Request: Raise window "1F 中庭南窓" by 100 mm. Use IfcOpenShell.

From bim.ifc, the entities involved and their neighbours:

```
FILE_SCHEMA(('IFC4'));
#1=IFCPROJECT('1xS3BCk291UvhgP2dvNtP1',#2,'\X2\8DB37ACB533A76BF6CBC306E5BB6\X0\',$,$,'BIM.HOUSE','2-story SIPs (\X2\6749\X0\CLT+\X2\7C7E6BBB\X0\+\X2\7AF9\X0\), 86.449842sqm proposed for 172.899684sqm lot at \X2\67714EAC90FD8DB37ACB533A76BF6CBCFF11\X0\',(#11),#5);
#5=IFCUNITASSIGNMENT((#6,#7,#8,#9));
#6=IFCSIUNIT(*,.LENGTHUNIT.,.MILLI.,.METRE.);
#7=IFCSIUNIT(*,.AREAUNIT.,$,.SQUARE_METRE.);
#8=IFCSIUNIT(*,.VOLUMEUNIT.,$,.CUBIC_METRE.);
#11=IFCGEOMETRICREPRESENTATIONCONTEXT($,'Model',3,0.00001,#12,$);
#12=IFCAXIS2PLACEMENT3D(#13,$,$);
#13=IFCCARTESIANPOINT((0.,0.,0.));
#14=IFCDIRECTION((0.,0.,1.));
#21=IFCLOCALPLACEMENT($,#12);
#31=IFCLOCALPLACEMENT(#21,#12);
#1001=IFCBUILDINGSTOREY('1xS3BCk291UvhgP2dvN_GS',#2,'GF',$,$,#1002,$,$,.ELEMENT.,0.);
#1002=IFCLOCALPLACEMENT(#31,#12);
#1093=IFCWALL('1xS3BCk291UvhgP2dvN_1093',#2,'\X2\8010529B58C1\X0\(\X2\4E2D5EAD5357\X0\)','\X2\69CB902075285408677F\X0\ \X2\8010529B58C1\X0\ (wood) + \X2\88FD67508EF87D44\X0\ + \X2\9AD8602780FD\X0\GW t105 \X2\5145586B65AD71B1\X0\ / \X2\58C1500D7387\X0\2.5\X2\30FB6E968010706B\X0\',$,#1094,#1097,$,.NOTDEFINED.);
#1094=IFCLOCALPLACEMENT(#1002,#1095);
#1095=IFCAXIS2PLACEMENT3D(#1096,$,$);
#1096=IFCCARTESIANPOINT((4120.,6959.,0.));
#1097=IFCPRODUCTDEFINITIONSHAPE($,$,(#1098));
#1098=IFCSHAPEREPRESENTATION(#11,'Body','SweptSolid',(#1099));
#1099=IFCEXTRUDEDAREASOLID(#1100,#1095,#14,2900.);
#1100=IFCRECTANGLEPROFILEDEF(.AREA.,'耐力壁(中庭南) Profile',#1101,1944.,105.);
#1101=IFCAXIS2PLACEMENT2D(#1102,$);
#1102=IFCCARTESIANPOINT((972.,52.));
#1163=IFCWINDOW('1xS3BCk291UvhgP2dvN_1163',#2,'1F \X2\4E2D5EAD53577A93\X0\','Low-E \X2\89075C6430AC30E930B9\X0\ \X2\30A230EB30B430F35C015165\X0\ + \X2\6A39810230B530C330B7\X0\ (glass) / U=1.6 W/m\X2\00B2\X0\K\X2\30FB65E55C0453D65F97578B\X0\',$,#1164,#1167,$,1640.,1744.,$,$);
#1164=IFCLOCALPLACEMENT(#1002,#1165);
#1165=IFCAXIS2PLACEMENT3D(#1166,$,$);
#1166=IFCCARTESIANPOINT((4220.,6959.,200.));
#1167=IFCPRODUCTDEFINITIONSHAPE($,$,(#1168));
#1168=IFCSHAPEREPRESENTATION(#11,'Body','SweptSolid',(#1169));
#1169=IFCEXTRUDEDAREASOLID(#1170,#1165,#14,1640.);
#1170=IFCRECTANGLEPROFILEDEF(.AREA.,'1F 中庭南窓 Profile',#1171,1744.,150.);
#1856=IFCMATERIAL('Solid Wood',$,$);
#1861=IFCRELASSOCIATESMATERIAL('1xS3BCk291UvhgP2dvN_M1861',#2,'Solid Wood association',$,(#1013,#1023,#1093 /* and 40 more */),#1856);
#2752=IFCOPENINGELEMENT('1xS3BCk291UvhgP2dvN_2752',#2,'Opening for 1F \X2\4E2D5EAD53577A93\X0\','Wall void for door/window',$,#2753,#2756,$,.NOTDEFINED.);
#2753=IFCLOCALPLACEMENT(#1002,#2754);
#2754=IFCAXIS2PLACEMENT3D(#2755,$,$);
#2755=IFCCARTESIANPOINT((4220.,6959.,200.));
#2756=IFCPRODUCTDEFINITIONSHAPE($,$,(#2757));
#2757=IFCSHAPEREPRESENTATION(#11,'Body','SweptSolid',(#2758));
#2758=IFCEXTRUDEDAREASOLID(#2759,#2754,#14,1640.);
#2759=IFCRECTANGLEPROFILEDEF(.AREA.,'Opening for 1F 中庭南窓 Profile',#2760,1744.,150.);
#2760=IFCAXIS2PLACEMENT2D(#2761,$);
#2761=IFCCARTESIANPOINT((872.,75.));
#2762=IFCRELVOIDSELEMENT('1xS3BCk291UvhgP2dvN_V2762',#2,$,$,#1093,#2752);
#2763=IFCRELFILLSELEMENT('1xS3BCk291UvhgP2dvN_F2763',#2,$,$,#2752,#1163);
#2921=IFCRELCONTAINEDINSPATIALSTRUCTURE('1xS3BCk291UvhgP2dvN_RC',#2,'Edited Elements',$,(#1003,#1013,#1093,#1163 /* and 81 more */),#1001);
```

```python
import numpy as np
import ifcopenshell
import ifcopenshell.api.geometry
import ifcopenshell.util.placement
import ifcopenshell.util.unit

model = ifcopenshell.open("bim.ifc")
unit_scale = ifcopenshell.util.unit.calculate_unit_scale(model)

window = model.by_guid("1xS3BCk291UvhgP2dvN_1163")
opening = window.FillsVoids[0].RelatingOpeningElement
dz = 100.0

shift = np.array([0.0, 0.0, dz])
# The window is not placed relative to its opening, so move both.
for product in (opening, window):
    matrix = ifcopenshell.util.placement.get_local_placement(product.ObjectPlacement)
    matrix[:3, 3] += shift
    ifcopenshell.api.geometry.edit_object_placement(model, product=product, matrix=matrix, is_si=False)

print(f"moved by {dz * unit_scale:+.3f} m")

model.write("bim-out.ifc")
```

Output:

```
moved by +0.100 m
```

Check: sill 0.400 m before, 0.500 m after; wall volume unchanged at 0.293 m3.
